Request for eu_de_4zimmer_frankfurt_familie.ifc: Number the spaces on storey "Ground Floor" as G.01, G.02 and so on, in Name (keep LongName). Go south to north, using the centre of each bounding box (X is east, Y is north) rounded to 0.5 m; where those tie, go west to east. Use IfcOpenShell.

First a look at what the model holds.

```python
import ifcopenshell
import ifcopenshell.util.element
import ifcopenshell.util.placement

model = ifcopenshell.open("eu_de_4zimmer_frankfurt_familie.ifc")
print(model.schema)
storey = next(s for s in model.by_type("IfcBuildingStorey") if s.Name == "Ground Floor")
spaces = [e for e in ifcopenshell.util.element.get_decomposition(storey) if e.is_a("IfcSpace")]
for e in sorted(spaces, key=lambda e: e.id()):
    origin = ifcopenshell.util.placement.get_local_placement(e.ObjectPlacement)[:3, 3]
    print(e.id(), e.Name, e.LongName, origin.round(2) + 0.0, sep=" | ")
```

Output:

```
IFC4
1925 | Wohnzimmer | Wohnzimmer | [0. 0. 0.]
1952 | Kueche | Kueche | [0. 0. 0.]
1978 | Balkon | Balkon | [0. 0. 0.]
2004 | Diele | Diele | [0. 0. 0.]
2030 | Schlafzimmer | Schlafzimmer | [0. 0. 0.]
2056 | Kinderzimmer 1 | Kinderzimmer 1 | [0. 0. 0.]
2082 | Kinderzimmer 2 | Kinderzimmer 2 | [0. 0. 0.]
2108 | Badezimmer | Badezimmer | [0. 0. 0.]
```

```python
import ifcopenshell
import ifcopenshell.geom
import ifcopenshell.util.element
import ifcopenshell.util.shape

model = ifcopenshell.open("eu_de_4zimmer_frankfurt_familie.ifc")
settings = ifcopenshell.geom.settings()
settings.set("use-world-coords", True)


def centre(element):
    shape = ifcopenshell.geom.create_shape(settings, element)
    return ifcopenshell.util.shape.get_bbox_centroid(shape.geometry)


storey = next(s for s in model.by_type("IfcBuildingStorey") if s.Name == "Ground Floor")
spaces = [e for e in ifcopenshell.util.element.get_decomposition(storey) if e.is_a("IfcSpace")]

# Insertion points can sit at a corner or the storey origin, so sort by the geometry (in metres).
centres = {e: centre(e) for e in spaces}
spaces.sort(key=lambda e: (round(centres[e][1] / 0.5), centres[e][0]))

for i, e in enumerate(spaces, start=1):
    number = f"G.{i:02d}"
    e.Name = number
    print(e.id(), number)

model.write("eu_de_4zimmer_frankfurt_familie-out.ifc")
```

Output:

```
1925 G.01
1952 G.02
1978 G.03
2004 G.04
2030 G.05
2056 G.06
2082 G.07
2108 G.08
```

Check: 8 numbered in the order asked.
